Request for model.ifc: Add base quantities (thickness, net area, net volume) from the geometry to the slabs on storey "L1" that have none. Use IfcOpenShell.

First a look at what the model holds.

```python
import ifcopenshell
import ifcopenshell.util.element
import ifcopenshell.util.unit

model = ifcopenshell.open("model.ifc")
print(model.schema)
for unit_type in ("LENGTHUNIT", "AREAUNIT", "VOLUMEUNIT"):
    print(unit_type, ifcopenshell.util.unit.calculate_unit_scale(model, unit_type))
storey = next(s for s in model.by_type("IfcBuildingStorey") if s.Name == "L1")
slabs = [e for e in ifcopenshell.util.element.get_decomposition(storey) if e.is_a("IfcSlab")]
for e in sorted(slabs, key=lambda e: e.id()):
    print(e.id(), e.is_a(), e.Name, list(ifcopenshell.util.element.get_psets(e, qtos_only=True)), sep=" | ")
```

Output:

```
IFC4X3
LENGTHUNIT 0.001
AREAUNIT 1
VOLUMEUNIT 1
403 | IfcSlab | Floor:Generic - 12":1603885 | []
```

```python
import ifcopenshell
import ifcopenshell.api.pset
import ifcopenshell.geom
import ifcopenshell.util.element
import ifcopenshell.util.shape
import ifcopenshell.util.unit

model = ifcopenshell.open("model.ifc")
unit_scale = ifcopenshell.util.unit.calculate_unit_scale(model)
area_scale = ifcopenshell.util.unit.calculate_unit_scale(model, "AREAUNIT")
volume_scale = ifcopenshell.util.unit.calculate_unit_scale(model, "VOLUMEUNIT")
settings = ifcopenshell.geom.settings()

storey = next(s for s in model.by_type("IfcBuildingStorey") if s.Name == "L1")
slabs = [e for e in ifcopenshell.util.element.get_decomposition(storey) if e.is_a("IfcSlab")]

for e in sorted(slabs, key=lambda e: e.id()):
    if ifcopenshell.util.element.get_psets(e, qtos_only=True, should_inherit=False):
        continue
    # Geometry comes back in metres, in the element's own axes.
    shape = ifcopenshell.geom.create_shape(settings, e)
    values = {
        "Width": ifcopenshell.util.shape.get_z(shape.geometry) / unit_scale,
        "NetArea": ifcopenshell.util.shape.get_footprint_area(shape.geometry) / area_scale,
        "NetVolume": ifcopenshell.util.shape.get_volume(shape.geometry) / volume_scale,
    }
    qto = ifcopenshell.api.pset.add_qto(model, product=e, name="Qto_SlabBaseQuantities")
    ifcopenshell.api.pset.edit_qto(model, qto=qto, properties=values)
    print(e.id(), {k: round(v, 3) for k, v in values.items()})

model.write("model_rev.ifc")
```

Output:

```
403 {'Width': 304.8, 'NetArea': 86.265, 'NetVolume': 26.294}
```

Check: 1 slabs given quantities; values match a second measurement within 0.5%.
